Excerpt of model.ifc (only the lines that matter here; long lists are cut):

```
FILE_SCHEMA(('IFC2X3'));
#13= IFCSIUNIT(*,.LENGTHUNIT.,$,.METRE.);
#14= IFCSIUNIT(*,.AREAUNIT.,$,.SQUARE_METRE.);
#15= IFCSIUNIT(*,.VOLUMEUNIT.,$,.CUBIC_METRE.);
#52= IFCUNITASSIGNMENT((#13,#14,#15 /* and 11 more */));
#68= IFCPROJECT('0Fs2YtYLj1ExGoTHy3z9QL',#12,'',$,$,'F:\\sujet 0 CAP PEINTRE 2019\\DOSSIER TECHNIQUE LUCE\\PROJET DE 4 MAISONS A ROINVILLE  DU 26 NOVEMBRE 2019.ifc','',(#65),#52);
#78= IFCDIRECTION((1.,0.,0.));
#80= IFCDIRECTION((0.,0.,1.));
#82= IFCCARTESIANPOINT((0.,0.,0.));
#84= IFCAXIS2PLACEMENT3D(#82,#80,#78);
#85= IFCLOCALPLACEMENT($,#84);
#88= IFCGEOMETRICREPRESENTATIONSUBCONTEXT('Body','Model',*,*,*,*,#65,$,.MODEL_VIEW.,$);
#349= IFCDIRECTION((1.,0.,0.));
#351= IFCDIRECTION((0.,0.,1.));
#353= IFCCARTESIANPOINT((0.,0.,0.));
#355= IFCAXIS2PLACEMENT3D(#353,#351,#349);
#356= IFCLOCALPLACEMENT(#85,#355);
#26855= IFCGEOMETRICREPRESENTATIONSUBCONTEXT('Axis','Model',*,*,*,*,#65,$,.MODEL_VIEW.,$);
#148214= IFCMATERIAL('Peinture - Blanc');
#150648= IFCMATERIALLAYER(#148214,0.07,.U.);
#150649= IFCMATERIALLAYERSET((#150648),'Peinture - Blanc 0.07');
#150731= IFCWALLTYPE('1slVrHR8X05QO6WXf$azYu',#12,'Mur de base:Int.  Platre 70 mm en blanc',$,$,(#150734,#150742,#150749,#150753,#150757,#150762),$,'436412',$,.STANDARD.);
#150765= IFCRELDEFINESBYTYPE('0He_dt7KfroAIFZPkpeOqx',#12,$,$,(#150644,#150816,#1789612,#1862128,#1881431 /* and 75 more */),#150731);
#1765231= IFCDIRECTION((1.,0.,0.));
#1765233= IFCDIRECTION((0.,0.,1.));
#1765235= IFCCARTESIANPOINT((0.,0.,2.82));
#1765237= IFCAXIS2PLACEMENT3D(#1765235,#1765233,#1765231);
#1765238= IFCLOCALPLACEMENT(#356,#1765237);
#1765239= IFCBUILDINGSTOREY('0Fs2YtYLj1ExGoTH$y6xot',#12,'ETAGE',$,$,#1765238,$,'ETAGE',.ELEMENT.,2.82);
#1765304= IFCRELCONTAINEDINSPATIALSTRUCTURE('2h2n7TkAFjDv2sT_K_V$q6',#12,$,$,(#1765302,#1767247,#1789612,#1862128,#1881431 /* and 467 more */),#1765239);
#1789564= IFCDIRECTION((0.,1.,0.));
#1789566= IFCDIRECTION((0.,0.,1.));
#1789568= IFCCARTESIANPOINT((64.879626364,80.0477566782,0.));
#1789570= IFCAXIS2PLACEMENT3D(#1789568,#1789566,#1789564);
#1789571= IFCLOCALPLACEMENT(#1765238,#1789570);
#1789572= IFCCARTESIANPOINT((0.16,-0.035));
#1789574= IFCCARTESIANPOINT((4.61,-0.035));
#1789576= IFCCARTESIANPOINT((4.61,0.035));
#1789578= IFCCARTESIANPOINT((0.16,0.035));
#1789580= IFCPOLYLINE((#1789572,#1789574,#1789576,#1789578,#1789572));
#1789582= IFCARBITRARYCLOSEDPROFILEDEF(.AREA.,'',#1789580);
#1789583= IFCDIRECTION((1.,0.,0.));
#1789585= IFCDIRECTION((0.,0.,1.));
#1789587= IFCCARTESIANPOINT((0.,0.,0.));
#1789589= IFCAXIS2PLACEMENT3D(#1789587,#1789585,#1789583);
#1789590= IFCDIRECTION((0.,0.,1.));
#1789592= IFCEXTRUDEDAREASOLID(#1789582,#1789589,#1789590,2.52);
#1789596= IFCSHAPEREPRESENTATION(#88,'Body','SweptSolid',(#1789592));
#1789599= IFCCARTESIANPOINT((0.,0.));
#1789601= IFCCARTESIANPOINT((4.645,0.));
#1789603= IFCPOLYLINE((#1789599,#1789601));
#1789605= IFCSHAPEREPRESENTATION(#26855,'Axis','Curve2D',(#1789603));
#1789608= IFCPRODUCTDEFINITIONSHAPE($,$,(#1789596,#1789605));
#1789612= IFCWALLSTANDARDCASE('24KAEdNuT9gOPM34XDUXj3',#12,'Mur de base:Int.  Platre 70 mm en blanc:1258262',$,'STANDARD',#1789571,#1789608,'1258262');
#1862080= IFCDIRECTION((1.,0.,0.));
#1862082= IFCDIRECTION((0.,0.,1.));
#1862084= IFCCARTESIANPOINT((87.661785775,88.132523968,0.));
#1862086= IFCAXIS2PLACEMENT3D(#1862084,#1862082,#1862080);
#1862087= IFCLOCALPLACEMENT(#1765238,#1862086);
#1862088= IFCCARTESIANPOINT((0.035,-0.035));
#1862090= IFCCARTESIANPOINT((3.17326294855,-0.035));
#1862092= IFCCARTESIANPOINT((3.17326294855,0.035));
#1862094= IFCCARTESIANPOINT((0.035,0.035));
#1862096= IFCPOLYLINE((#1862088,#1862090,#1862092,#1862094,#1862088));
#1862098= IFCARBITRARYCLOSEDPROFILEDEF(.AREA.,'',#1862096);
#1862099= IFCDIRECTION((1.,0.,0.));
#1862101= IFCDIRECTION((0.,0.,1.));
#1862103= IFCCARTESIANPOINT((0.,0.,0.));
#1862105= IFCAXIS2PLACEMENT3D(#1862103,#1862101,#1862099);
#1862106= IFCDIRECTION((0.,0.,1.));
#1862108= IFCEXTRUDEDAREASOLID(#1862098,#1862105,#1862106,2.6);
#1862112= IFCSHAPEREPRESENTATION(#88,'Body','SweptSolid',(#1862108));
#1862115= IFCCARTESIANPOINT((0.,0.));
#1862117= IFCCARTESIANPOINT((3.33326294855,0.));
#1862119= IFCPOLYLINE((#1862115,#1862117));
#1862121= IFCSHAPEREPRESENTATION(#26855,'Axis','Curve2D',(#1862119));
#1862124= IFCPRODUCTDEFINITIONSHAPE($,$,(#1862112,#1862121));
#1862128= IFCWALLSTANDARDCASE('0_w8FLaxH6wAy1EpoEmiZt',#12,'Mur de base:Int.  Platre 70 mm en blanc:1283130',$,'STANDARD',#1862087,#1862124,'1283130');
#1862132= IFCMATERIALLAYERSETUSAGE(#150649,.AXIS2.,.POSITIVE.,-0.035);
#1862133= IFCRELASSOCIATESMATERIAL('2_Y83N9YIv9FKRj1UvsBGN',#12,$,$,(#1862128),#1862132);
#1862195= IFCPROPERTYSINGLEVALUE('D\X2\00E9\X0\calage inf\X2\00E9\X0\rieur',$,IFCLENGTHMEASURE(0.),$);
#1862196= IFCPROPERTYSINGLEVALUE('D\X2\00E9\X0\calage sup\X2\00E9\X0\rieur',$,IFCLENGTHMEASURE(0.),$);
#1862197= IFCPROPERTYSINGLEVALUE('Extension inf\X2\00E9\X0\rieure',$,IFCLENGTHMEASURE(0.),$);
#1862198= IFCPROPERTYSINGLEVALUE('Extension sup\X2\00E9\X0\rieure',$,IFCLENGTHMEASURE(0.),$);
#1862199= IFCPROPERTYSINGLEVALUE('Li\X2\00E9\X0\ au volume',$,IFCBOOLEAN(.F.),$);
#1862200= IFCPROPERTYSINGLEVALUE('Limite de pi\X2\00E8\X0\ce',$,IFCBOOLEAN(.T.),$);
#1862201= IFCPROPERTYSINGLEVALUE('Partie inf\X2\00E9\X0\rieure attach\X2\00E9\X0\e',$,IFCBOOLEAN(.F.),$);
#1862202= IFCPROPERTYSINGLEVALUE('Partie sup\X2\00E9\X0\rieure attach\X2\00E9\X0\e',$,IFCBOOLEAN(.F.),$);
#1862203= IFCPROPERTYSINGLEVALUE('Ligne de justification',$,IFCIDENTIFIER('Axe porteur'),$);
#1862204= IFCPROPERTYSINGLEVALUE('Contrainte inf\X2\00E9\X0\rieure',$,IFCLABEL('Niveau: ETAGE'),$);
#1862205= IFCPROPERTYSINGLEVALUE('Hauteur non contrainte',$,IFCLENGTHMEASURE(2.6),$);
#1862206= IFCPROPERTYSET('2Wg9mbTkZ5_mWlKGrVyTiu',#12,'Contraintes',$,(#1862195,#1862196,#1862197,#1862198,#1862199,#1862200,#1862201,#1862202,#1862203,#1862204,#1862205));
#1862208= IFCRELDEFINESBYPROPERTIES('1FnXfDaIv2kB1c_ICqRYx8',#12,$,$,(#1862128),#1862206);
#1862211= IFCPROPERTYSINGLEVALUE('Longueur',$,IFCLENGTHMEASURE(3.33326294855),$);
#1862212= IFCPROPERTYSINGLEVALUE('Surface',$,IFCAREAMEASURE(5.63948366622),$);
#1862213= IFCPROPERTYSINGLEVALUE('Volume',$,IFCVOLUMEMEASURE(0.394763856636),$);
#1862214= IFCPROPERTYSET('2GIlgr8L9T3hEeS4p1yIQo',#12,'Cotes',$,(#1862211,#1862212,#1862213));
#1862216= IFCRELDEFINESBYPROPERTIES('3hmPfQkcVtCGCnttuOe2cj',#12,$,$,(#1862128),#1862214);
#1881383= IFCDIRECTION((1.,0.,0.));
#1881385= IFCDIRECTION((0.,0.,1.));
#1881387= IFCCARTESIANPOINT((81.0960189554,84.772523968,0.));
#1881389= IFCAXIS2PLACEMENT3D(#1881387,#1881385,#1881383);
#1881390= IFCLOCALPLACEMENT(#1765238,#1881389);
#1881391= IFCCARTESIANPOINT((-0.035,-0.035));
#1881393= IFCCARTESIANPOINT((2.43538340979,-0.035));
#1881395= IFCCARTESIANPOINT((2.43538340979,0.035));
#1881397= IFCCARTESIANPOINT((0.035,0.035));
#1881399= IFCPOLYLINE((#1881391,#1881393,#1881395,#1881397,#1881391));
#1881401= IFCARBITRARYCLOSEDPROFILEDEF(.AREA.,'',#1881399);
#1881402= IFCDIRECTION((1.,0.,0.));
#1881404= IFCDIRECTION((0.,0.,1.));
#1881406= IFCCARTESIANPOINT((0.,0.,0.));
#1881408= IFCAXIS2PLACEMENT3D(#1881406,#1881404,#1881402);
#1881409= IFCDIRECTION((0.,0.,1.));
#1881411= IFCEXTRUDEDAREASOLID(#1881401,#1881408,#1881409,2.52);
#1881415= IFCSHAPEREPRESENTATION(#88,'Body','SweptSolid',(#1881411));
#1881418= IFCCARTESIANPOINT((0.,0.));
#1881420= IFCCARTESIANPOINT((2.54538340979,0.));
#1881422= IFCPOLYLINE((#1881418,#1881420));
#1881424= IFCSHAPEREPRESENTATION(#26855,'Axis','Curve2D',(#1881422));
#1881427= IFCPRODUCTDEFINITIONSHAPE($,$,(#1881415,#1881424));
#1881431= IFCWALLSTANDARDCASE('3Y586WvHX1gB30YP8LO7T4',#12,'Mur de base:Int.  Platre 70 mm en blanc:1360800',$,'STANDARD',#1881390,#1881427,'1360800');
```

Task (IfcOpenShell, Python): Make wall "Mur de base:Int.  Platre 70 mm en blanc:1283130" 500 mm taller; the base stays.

```python
import ifcopenshell
import ifcopenshell.api.pset
import ifcopenshell.geom
import ifcopenshell.util.element
import ifcopenshell.util.representation
import ifcopenshell.util.shape
import ifcopenshell.util.unit

model = ifcopenshell.open("model.ifc")
unit_scale = ifcopenshell.util.unit.calculate_unit_scale(model)
area_scale = ifcopenshell.util.unit.calculate_unit_scale(model, "AREAUNIT")
volume_scale = ifcopenshell.util.unit.calculate_unit_scale(model, "VOLUMEUNIT")
settings = ifcopenshell.geom.settings()


def volume(element):
    """Net volume in cubic metres, openings subtracted."""
    shape = ifcopenshell.geom.create_shape(settings, element)
    return ifcopenshell.util.shape.get_volume(shape.geometry)


wall = model.by_guid("0_w8FLaxH6wAy1EpoEmiZt")
before = volume(wall)

body = ifcopenshell.util.representation.get_representation(wall, "Model", "Body")
solid = body.Items[0]
old_height = solid.Depth
solid.Depth += 0.5 / unit_scale
after = volume(wall)
thickness = 0.07  # wall thickness in metres

# Update the stored height, areas and volumes.
pset = model.by_id(ifcopenshell.util.element.get_pset(wall, "Contraintes", should_inherit=False)["id"])
ifcopenshell.api.pset.edit_pset(model, pset=pset, properties={
    "Hauteur non contrainte": model.create_entity("IfcLengthMeasure", solid.Depth),
})
pset = model.by_id(ifcopenshell.util.element.get_pset(wall, "Cotes", should_inherit=False)["id"])
ifcopenshell.api.pset.edit_pset(model, pset=pset, properties={
    "Surface": model.create_entity("IfcAreaMeasure", after / thickness / area_scale),
    "Volume": model.create_entity("IfcVolumeMeasure", after / volume_scale),
})

print(f"height {old_height:g} -> {solid.Depth:g}, volume {before:.3f} -> {after:.3f} m3")

model.write("model-out.ifc")
```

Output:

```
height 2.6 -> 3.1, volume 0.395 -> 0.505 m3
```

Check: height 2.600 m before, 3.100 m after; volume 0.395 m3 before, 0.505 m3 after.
